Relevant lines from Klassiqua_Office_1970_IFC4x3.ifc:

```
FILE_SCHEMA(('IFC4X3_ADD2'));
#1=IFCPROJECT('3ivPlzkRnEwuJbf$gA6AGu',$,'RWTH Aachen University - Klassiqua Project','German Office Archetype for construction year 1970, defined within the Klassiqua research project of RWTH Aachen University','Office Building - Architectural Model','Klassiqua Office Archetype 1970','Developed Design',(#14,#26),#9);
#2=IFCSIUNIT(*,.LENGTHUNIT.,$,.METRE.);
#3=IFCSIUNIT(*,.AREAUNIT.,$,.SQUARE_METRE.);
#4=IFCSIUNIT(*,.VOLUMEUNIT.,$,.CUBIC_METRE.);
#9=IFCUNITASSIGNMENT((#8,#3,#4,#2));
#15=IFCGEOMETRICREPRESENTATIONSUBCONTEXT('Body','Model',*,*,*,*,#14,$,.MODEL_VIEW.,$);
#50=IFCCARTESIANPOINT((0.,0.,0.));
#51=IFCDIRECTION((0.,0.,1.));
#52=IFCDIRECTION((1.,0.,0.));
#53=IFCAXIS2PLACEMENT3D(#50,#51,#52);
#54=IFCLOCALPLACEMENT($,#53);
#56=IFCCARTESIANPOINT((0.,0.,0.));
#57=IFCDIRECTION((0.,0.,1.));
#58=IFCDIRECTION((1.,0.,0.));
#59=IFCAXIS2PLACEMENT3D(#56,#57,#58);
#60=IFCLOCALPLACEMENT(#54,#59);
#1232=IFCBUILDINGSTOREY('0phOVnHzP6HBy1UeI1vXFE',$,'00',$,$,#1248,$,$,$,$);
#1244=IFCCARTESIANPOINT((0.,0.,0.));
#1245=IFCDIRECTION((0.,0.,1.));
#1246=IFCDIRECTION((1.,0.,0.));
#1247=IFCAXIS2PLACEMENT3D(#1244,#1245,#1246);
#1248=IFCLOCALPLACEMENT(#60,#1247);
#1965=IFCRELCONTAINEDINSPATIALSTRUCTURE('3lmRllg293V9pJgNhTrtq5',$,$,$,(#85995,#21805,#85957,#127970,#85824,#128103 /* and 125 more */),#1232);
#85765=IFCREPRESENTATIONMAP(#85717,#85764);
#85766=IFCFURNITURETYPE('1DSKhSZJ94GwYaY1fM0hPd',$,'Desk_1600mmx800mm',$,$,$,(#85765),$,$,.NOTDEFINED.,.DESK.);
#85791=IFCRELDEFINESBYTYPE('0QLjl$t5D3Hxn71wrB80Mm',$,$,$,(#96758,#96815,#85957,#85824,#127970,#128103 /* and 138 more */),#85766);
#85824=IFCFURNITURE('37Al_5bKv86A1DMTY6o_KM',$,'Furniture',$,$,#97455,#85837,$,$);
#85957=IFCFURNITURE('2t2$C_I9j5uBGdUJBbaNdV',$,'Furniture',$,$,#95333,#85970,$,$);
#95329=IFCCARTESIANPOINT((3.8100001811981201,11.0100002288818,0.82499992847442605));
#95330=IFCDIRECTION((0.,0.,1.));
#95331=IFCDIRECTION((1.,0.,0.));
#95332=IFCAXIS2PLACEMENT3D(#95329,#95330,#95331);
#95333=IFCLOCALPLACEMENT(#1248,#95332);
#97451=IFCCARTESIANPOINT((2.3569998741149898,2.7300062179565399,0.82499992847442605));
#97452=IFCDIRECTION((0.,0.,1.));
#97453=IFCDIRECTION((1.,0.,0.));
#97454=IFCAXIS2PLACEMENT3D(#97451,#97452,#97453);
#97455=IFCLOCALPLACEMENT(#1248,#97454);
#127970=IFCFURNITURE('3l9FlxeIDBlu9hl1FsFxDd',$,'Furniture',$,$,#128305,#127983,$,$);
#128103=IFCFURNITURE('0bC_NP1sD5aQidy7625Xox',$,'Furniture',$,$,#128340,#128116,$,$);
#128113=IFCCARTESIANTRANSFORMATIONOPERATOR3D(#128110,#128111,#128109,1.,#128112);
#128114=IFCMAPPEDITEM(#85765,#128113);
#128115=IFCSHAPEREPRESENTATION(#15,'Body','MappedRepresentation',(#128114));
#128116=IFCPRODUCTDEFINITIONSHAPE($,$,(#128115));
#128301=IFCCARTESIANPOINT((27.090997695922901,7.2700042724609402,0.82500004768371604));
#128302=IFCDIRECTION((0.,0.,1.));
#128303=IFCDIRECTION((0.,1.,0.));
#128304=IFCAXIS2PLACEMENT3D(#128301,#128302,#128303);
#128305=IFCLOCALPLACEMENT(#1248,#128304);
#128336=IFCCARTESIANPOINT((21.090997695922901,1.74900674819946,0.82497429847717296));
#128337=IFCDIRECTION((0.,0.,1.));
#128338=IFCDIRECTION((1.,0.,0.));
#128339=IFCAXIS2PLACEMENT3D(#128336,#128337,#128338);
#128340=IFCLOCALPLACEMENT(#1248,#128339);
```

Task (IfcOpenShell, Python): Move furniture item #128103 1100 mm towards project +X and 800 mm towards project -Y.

```python
import ifcopenshell
import ifcopenshell.api.geometry
import ifcopenshell.util.placement

model = ifcopenshell.open("Klassiqua_Office_1970_IFC4x3.ifc")

item = model.by_guid("0bC_NP1sD5aQidy7625Xox")
matrix = ifcopenshell.util.placement.get_local_placement(item.ObjectPlacement)
matrix[0, 3] += 1.1
matrix[1, 3] -= 0.8
ifcopenshell.api.geometry.edit_object_placement(model, product=item, matrix=matrix, is_si=False)

print(ifcopenshell.util.placement.get_local_placement(item.ObjectPlacement).round(3) + 0.0)

model.write("Klassiqua_Office_1970_IFC4x3_rev.ifc")
```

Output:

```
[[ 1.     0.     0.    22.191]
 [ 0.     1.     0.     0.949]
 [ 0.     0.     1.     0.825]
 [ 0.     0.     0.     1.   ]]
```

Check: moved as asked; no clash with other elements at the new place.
